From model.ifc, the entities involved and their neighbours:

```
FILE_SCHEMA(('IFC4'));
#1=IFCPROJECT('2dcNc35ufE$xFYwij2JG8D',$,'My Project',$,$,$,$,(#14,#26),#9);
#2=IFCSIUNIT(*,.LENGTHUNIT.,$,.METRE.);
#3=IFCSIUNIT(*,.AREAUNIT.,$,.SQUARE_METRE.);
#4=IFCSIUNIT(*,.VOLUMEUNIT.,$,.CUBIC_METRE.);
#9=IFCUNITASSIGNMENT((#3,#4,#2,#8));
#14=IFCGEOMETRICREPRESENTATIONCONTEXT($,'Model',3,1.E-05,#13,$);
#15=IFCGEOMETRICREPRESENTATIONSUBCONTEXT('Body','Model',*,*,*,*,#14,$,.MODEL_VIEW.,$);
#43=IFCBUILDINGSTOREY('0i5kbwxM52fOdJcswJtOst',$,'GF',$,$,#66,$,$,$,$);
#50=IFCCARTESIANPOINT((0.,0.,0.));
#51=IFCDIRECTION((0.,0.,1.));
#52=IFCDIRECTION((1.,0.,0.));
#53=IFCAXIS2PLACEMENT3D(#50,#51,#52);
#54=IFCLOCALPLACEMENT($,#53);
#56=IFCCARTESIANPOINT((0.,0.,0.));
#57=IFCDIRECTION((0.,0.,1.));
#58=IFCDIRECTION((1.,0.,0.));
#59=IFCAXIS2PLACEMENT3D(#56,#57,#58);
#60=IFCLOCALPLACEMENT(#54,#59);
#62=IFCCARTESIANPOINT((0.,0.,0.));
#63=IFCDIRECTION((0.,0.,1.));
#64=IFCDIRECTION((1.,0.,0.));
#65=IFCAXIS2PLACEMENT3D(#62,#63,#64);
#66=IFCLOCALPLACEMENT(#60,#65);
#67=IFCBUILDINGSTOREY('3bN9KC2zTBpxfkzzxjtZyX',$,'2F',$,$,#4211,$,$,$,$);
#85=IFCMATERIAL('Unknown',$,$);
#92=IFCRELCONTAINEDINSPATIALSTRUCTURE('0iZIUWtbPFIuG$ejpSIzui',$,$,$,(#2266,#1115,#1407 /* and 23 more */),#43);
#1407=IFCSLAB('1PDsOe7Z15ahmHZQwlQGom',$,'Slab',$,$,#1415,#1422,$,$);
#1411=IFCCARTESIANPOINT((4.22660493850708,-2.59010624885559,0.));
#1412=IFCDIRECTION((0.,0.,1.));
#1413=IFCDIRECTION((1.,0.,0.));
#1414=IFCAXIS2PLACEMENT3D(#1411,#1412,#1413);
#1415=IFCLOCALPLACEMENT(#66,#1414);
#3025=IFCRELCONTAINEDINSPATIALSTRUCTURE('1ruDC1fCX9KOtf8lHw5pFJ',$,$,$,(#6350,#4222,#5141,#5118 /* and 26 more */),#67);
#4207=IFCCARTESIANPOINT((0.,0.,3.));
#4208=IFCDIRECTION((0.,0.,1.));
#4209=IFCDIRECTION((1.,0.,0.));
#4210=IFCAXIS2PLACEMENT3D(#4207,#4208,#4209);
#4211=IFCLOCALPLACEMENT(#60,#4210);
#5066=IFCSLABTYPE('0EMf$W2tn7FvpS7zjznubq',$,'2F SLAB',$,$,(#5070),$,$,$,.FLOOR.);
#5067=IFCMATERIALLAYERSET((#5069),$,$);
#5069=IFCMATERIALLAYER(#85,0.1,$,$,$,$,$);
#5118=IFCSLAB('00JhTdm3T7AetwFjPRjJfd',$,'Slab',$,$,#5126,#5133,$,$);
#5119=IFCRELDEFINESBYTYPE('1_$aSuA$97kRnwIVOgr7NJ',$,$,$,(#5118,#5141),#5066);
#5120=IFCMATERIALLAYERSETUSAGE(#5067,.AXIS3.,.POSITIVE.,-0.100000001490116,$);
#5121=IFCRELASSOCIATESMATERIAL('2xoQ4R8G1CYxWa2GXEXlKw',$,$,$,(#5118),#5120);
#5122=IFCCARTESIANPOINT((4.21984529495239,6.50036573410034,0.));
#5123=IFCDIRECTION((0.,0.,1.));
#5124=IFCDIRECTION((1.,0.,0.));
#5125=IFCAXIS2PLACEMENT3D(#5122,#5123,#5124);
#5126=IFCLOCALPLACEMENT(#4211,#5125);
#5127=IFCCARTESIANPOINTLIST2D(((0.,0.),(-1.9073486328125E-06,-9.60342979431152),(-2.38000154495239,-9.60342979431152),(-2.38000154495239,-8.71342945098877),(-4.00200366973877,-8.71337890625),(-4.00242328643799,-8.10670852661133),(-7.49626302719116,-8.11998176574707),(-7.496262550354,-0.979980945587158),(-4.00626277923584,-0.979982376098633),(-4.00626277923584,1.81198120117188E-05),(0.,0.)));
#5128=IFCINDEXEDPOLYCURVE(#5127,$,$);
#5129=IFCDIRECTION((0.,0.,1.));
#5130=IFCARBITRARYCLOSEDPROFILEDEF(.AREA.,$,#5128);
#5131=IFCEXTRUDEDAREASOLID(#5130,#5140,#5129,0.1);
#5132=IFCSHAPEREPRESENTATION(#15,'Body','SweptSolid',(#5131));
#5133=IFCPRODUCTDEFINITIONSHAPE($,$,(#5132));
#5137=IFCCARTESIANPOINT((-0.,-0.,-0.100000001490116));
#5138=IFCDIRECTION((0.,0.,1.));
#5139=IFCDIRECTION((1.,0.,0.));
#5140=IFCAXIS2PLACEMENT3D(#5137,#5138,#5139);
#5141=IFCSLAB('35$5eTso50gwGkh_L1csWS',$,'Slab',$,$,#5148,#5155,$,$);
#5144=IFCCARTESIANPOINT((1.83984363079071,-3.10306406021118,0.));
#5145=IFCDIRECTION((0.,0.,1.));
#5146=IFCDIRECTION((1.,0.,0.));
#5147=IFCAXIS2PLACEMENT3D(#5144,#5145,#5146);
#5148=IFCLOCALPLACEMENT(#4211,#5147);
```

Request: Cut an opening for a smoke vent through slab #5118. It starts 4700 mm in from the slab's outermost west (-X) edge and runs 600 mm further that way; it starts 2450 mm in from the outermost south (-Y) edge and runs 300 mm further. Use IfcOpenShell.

```python
import numpy as np
import ifcopenshell
import ifcopenshell.api.feature
import ifcopenshell.api.geometry
import ifcopenshell.api.root
import ifcopenshell.geom
import ifcopenshell.util.placement
import ifcopenshell.util.representation
import ifcopenshell.util.shape
import ifcopenshell.util.unit

model = ifcopenshell.open("model.ifc")
unit_scale = ifcopenshell.util.unit.calculate_unit_scale(model)
settings = ifcopenshell.geom.settings()


def volume(element):
    """Net volume in cubic metres, openings subtracted."""
    shape = ifcopenshell.geom.create_shape(settings, element)
    return ifcopenshell.util.shape.get_volume(shape.geometry)


slab = model.by_guid("00JhTdm3T7AetwFjPRjJfd")
before = volume(slab)

# Extent in the slab's own axes, in metres. The edges named are its -X and -Y sides.
slab_shape = ifcopenshell.geom.create_shape(settings, slab)
vertices = ifcopenshell.util.shape.get_vertices(slab_shape.geometry)
x_min, y_min, bottom = vertices.min(axis=0)
top = vertices[:, 2].max()

opening = ifcopenshell.api.root.create_entity(model, ifc_class="IfcOpeningElement", name="Smoke vent opening", predefined_type="OPENING")
context = ifcopenshell.util.representation.get_context(model, "Model", "Body", "MODEL_VIEW")
width, depth = 0.6, 0.3
outline = [(0.0, 0.0), (width, 0.0), (width, depth), (0.0, depth), (0.0, 0.0)]
# Overshoot both faces by 50 mm so the cut is clean.
shape = ifcopenshell.api.geometry.add_slab_representation(
    model, context=context, depth=top - bottom + 0.1, polyline=outline
)
ifcopenshell.api.geometry.assign_representation(model, product=opening, representation=shape)

matrix = ifcopenshell.util.placement.get_local_placement(slab.ObjectPlacement)
matrix[:, 3] = matrix @ np.append(np.array([x_min + 4.7, y_min + 2.45, bottom - 0.05]) / unit_scale, 1.0)
ifcopenshell.api.geometry.edit_object_placement(model, product=opening, matrix=matrix, is_si=False)
ifcopenshell.api.feature.add_feature(model, feature=opening, element=slab)

after = volume(slab)

print(f"slab volume {before:.3f} -> {after:.3f} m3")

model.write("model-out.ifc")
```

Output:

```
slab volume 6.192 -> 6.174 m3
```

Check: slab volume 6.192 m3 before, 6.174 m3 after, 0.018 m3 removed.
